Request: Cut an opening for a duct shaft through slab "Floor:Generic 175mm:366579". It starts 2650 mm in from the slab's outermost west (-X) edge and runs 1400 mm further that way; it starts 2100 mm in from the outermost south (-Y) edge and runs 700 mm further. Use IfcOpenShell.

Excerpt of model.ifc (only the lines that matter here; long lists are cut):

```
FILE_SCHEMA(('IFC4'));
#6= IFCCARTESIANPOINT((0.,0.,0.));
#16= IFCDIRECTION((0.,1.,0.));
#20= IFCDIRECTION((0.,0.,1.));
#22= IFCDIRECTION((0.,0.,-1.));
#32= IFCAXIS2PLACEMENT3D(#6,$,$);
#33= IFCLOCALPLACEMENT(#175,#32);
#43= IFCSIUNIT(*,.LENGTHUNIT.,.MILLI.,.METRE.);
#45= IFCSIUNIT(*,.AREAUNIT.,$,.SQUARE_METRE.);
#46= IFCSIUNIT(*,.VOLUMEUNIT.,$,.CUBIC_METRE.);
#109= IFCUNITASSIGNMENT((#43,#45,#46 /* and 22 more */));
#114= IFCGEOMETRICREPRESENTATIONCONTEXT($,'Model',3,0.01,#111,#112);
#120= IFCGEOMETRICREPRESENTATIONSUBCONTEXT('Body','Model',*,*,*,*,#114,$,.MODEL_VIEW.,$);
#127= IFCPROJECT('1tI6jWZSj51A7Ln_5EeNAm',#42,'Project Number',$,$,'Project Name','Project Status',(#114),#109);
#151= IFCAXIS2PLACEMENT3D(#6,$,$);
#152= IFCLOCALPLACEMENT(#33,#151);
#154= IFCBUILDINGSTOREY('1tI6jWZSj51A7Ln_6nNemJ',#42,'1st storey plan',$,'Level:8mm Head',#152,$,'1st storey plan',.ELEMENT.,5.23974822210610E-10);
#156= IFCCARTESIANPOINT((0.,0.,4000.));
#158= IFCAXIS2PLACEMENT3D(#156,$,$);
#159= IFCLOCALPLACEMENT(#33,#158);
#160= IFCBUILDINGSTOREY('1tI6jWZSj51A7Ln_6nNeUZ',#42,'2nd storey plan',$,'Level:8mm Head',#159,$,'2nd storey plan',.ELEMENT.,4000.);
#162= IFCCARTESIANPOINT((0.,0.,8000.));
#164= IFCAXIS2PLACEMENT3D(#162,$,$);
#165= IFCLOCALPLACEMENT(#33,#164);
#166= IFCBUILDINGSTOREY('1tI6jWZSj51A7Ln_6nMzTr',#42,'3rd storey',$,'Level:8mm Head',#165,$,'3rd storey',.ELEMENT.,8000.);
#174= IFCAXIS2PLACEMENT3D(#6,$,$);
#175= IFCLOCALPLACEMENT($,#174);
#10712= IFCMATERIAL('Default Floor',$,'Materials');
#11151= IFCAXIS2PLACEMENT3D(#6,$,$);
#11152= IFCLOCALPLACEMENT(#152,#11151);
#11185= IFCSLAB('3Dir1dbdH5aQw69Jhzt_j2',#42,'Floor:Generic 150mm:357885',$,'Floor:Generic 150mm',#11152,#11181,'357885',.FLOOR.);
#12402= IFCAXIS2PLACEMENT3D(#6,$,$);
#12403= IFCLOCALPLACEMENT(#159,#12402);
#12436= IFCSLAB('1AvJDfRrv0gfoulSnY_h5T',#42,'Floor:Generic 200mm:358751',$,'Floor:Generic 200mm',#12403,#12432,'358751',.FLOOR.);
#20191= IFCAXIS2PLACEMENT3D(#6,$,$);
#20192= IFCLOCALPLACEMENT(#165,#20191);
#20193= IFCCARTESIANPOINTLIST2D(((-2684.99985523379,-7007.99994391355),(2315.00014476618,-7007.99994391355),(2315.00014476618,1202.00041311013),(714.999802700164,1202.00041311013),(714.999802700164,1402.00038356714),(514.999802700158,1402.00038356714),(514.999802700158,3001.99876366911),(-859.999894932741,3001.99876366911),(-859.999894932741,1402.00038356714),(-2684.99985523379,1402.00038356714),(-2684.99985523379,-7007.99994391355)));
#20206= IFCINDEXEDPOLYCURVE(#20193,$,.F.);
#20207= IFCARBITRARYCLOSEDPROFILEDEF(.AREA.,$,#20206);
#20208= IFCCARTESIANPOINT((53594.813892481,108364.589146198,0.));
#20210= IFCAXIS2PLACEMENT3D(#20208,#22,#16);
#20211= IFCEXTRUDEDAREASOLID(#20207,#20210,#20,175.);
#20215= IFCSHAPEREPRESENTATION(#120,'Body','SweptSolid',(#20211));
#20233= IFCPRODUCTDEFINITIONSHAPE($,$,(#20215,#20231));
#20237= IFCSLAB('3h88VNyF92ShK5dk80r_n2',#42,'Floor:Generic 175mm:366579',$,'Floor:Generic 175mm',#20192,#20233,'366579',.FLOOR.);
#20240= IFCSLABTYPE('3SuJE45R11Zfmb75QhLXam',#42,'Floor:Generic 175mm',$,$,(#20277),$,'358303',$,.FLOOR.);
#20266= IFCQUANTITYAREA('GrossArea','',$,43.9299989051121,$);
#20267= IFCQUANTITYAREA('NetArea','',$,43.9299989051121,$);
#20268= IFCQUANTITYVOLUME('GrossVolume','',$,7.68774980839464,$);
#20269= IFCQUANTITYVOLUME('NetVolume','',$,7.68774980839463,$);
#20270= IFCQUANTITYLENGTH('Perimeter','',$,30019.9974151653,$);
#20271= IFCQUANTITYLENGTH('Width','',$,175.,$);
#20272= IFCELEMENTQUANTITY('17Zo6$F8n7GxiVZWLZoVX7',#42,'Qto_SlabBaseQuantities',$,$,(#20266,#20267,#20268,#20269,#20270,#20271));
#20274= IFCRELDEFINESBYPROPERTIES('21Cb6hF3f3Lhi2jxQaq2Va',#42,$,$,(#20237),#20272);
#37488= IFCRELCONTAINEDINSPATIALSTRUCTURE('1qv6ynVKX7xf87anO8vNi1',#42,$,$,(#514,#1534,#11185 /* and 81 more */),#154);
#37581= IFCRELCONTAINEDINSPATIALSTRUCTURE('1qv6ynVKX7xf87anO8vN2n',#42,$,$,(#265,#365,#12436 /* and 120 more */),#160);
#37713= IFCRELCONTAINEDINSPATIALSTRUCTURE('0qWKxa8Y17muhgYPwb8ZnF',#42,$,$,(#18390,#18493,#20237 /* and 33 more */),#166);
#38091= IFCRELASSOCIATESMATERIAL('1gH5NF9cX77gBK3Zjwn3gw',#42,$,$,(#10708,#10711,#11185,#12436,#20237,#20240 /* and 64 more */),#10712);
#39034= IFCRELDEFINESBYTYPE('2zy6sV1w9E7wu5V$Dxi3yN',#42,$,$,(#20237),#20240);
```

```python
import numpy as np
import ifcopenshell
import ifcopenshell.api.feature
import ifcopenshell.api.geometry
import ifcopenshell.api.pset
import ifcopenshell.api.root
import ifcopenshell.geom
import ifcopenshell.util.element
import ifcopenshell.util.placement
import ifcopenshell.util.representation
import ifcopenshell.util.shape
import ifcopenshell.util.unit

model = ifcopenshell.open("model.ifc")
unit_scale = ifcopenshell.util.unit.calculate_unit_scale(model)
area_scale = ifcopenshell.util.unit.calculate_unit_scale(model, "AREAUNIT")
volume_scale = ifcopenshell.util.unit.calculate_unit_scale(model, "VOLUMEUNIT")
settings = ifcopenshell.geom.settings()


def volume(element):
    """Net volume in cubic metres, openings subtracted."""
    shape = ifcopenshell.geom.create_shape(settings, element)
    return ifcopenshell.util.shape.get_volume(shape.geometry)


slab = model.by_guid("3h88VNyF92ShK5dk80r_n2")
before = volume(slab)

# Extent in the slab's own axes, in metres. The edges named are its -X and -Y sides.
slab_shape = ifcopenshell.geom.create_shape(settings, slab)
vertices = ifcopenshell.util.shape.get_vertices(slab_shape.geometry)
x_min, y_min, bottom = vertices.min(axis=0)
top = vertices[:, 2].max()

opening = ifcopenshell.api.root.create_entity(model, ifc_class="IfcOpeningElement", name="Duct shaft opening", predefined_type="OPENING")
context = ifcopenshell.util.representation.get_context(model, "Model", "Body", "MODEL_VIEW")
width, depth = 1.4, 0.7
outline = [(0.0, 0.0), (width, 0.0), (width, depth), (0.0, depth), (0.0, 0.0)]
# Overshoot both faces by 50 mm so the cut is clean.
shape = ifcopenshell.api.geometry.add_slab_representation(
    model, context=context, depth=top - bottom + 0.1, polyline=outline
)
ifcopenshell.api.geometry.assign_representation(model, product=opening, representation=shape)

matrix = ifcopenshell.util.placement.get_local_placement(slab.ObjectPlacement)
matrix[:, 3] = matrix @ np.append(np.array([x_min + 2.65, y_min + 2.1, bottom - 0.05]) / unit_scale, 1.0)
ifcopenshell.api.geometry.edit_object_placement(model, product=opening, matrix=matrix, is_si=False)
ifcopenshell.api.feature.add_feature(model, feature=opening, element=slab)

after = volume(slab)

# Update the slab's stored quantities.
qto = model.by_id(ifcopenshell.util.element.get_pset(slab, "Qto_SlabBaseQuantities", should_inherit=False)["id"])
ifcopenshell.api.pset.edit_qto(model, qto=qto, properties={
    "NetArea": after / (top - bottom) / area_scale,
    "NetVolume": after / volume_scale,
})

print(f"slab volume {before:.3f} -> {after:.3f} m3")

model.write("model_updated.ifc")
```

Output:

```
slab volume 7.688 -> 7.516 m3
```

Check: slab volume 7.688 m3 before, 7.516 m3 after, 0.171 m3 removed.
